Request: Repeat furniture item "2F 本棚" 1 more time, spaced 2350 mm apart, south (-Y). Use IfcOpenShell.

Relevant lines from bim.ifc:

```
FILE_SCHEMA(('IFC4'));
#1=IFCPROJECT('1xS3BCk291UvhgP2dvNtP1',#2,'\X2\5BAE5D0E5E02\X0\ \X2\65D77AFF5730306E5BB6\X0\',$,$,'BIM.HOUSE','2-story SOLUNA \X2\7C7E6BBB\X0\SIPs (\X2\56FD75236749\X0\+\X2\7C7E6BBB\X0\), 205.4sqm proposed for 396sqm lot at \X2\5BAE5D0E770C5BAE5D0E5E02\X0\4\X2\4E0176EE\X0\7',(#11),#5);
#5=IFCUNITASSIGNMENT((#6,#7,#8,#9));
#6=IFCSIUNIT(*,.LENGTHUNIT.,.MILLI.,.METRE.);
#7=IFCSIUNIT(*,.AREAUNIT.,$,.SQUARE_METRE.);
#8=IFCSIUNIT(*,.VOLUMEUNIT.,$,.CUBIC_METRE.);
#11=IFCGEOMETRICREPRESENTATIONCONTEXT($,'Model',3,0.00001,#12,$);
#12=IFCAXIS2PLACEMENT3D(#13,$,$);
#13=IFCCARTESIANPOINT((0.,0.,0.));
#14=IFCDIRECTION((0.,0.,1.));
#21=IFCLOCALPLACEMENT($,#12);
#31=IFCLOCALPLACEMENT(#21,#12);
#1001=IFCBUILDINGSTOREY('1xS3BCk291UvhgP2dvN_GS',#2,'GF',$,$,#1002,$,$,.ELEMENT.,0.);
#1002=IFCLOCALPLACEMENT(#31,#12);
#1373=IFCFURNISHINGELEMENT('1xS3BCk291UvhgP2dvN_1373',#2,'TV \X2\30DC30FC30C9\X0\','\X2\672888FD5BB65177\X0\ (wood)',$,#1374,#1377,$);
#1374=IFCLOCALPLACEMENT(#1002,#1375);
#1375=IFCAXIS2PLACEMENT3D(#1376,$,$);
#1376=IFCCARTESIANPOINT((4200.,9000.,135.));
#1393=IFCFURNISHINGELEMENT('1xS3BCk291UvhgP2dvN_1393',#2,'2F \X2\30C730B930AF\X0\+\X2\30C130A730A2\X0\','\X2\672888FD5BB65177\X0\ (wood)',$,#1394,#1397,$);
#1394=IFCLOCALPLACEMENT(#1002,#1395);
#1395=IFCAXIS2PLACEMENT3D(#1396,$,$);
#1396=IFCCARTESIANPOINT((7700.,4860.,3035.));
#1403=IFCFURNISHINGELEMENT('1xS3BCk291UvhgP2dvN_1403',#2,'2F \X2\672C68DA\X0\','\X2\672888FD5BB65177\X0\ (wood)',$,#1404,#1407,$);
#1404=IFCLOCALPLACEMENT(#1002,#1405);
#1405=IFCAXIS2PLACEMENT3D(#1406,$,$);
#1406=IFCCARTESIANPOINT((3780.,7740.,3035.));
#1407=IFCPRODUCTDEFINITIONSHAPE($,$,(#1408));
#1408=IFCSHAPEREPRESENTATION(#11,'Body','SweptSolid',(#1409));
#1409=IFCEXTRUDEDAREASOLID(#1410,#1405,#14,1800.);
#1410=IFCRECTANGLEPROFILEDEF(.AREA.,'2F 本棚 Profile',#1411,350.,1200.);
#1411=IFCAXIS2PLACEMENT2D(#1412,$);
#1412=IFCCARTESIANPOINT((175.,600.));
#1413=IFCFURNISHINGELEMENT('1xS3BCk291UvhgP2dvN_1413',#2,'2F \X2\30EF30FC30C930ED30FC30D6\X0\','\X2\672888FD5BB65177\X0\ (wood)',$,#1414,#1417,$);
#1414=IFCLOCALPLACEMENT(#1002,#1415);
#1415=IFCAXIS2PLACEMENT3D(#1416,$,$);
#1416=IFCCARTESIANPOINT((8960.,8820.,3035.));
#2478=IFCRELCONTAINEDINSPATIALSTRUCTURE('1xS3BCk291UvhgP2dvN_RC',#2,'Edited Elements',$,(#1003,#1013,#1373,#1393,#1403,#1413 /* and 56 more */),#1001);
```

```python
import numpy as np
import ifcopenshell
import ifcopenshell.api.geometry
import ifcopenshell.api.root
import ifcopenshell.util.element
import ifcopenshell.util.placement

model = ifcopenshell.open("bim.ifc")


def reuse_history(source, copy):
    """copy_class also copies each property set's owner history, people and application; keep the originals."""
    for rel in copy.IsDefinedBy:
        if rel.is_a("IfcRelDefinesByProperties") and (history := rel.RelatingPropertyDefinition.OwnerHistory):
            rel.RelatingPropertyDefinition.OwnerHistory = source.OwnerHistory
            ifcopenshell.util.element.remove_deep2(model, history)


source = model.by_guid("1xS3BCk291UvhgP2dvN_1403")
base = ifcopenshell.util.placement.get_local_placement(source.ObjectPlacement)
step = np.array([0.0, -1.0, 0.0]) * 2350.0

for i in range(1, 2):
    copy = ifcopenshell.api.root.copy_class(model, product=source)
    copy.Representation = ifcopenshell.util.element.copy_deep(
        model, source.Representation, exclude=["IfcGeometricRepresentationContext", "IfcRepresentationMap"]
    )
    reuse_history(source, copy)
    matrix = base.copy()
    matrix[:3, 3] += i * step
    print("added at", matrix[:3, 3].round(3) + 0.0)
    ifcopenshell.api.geometry.edit_object_placement(model, product=copy, matrix=matrix, is_si=False)

model.write("bim_rev.ifc")
```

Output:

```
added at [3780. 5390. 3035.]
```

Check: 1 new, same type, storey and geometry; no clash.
